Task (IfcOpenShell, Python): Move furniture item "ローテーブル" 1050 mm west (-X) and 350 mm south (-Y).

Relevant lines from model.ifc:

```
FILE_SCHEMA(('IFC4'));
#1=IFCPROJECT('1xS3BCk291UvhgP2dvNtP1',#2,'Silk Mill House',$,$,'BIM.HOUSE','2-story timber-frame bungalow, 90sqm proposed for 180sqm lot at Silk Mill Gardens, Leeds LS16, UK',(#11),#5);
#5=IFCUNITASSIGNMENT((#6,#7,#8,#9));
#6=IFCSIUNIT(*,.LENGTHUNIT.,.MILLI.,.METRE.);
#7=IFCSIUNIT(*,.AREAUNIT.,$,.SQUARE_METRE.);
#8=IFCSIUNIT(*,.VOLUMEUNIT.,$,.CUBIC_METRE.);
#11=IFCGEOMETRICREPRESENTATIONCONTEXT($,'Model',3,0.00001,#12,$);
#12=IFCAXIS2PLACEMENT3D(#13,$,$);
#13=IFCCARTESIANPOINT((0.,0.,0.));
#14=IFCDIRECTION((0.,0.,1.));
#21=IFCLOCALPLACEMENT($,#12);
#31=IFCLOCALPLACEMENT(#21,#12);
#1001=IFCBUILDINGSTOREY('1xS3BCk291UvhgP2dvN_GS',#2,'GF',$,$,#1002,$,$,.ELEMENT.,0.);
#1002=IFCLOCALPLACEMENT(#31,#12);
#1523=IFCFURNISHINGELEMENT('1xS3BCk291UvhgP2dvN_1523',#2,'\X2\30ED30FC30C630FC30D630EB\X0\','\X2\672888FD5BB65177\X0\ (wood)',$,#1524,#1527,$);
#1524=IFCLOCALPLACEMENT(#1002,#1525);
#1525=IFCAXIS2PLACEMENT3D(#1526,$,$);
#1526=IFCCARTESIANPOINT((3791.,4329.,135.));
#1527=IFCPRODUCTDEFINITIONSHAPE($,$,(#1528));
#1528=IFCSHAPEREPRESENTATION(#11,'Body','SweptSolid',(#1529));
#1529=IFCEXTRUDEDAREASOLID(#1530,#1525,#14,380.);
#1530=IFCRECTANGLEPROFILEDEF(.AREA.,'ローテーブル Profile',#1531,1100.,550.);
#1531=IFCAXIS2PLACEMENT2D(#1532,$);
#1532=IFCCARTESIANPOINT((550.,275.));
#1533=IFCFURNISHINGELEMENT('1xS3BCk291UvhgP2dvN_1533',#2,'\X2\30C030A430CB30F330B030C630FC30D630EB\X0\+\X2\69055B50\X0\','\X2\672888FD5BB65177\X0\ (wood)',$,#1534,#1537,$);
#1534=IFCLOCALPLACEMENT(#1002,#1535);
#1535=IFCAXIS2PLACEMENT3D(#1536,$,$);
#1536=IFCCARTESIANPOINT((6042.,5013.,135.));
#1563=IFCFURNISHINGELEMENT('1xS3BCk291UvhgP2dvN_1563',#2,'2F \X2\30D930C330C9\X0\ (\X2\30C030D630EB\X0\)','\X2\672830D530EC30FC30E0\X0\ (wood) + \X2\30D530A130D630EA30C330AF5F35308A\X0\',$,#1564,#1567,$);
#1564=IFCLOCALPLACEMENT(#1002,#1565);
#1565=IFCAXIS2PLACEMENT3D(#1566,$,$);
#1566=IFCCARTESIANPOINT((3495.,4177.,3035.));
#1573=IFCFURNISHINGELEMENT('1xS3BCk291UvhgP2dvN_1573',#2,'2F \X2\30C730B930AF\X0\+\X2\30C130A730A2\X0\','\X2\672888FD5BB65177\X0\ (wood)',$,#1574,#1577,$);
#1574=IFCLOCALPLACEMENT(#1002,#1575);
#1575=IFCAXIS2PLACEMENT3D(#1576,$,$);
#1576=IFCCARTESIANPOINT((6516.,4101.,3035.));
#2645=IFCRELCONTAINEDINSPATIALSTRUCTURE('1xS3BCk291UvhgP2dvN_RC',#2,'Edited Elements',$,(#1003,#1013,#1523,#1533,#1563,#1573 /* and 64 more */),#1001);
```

```python
import ifcopenshell
import ifcopenshell.api.geometry
import ifcopenshell.util.placement

model = ifcopenshell.open("model.ifc")

item = model.by_guid("1xS3BCk291UvhgP2dvN_1523")
matrix = ifcopenshell.util.placement.get_local_placement(item.ObjectPlacement)
matrix[0, 3] -= 1050.0
matrix[1, 3] -= 350.0
ifcopenshell.api.geometry.edit_object_placement(model, product=item, matrix=matrix, is_si=False)

print(ifcopenshell.util.placement.get_local_placement(item.ObjectPlacement).round(3) + 0.0)

model.write("model_updated.ifc")
```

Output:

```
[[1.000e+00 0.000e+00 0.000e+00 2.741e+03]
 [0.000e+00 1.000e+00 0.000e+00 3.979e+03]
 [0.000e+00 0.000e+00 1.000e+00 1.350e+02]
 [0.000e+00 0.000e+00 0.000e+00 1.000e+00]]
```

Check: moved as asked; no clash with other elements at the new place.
